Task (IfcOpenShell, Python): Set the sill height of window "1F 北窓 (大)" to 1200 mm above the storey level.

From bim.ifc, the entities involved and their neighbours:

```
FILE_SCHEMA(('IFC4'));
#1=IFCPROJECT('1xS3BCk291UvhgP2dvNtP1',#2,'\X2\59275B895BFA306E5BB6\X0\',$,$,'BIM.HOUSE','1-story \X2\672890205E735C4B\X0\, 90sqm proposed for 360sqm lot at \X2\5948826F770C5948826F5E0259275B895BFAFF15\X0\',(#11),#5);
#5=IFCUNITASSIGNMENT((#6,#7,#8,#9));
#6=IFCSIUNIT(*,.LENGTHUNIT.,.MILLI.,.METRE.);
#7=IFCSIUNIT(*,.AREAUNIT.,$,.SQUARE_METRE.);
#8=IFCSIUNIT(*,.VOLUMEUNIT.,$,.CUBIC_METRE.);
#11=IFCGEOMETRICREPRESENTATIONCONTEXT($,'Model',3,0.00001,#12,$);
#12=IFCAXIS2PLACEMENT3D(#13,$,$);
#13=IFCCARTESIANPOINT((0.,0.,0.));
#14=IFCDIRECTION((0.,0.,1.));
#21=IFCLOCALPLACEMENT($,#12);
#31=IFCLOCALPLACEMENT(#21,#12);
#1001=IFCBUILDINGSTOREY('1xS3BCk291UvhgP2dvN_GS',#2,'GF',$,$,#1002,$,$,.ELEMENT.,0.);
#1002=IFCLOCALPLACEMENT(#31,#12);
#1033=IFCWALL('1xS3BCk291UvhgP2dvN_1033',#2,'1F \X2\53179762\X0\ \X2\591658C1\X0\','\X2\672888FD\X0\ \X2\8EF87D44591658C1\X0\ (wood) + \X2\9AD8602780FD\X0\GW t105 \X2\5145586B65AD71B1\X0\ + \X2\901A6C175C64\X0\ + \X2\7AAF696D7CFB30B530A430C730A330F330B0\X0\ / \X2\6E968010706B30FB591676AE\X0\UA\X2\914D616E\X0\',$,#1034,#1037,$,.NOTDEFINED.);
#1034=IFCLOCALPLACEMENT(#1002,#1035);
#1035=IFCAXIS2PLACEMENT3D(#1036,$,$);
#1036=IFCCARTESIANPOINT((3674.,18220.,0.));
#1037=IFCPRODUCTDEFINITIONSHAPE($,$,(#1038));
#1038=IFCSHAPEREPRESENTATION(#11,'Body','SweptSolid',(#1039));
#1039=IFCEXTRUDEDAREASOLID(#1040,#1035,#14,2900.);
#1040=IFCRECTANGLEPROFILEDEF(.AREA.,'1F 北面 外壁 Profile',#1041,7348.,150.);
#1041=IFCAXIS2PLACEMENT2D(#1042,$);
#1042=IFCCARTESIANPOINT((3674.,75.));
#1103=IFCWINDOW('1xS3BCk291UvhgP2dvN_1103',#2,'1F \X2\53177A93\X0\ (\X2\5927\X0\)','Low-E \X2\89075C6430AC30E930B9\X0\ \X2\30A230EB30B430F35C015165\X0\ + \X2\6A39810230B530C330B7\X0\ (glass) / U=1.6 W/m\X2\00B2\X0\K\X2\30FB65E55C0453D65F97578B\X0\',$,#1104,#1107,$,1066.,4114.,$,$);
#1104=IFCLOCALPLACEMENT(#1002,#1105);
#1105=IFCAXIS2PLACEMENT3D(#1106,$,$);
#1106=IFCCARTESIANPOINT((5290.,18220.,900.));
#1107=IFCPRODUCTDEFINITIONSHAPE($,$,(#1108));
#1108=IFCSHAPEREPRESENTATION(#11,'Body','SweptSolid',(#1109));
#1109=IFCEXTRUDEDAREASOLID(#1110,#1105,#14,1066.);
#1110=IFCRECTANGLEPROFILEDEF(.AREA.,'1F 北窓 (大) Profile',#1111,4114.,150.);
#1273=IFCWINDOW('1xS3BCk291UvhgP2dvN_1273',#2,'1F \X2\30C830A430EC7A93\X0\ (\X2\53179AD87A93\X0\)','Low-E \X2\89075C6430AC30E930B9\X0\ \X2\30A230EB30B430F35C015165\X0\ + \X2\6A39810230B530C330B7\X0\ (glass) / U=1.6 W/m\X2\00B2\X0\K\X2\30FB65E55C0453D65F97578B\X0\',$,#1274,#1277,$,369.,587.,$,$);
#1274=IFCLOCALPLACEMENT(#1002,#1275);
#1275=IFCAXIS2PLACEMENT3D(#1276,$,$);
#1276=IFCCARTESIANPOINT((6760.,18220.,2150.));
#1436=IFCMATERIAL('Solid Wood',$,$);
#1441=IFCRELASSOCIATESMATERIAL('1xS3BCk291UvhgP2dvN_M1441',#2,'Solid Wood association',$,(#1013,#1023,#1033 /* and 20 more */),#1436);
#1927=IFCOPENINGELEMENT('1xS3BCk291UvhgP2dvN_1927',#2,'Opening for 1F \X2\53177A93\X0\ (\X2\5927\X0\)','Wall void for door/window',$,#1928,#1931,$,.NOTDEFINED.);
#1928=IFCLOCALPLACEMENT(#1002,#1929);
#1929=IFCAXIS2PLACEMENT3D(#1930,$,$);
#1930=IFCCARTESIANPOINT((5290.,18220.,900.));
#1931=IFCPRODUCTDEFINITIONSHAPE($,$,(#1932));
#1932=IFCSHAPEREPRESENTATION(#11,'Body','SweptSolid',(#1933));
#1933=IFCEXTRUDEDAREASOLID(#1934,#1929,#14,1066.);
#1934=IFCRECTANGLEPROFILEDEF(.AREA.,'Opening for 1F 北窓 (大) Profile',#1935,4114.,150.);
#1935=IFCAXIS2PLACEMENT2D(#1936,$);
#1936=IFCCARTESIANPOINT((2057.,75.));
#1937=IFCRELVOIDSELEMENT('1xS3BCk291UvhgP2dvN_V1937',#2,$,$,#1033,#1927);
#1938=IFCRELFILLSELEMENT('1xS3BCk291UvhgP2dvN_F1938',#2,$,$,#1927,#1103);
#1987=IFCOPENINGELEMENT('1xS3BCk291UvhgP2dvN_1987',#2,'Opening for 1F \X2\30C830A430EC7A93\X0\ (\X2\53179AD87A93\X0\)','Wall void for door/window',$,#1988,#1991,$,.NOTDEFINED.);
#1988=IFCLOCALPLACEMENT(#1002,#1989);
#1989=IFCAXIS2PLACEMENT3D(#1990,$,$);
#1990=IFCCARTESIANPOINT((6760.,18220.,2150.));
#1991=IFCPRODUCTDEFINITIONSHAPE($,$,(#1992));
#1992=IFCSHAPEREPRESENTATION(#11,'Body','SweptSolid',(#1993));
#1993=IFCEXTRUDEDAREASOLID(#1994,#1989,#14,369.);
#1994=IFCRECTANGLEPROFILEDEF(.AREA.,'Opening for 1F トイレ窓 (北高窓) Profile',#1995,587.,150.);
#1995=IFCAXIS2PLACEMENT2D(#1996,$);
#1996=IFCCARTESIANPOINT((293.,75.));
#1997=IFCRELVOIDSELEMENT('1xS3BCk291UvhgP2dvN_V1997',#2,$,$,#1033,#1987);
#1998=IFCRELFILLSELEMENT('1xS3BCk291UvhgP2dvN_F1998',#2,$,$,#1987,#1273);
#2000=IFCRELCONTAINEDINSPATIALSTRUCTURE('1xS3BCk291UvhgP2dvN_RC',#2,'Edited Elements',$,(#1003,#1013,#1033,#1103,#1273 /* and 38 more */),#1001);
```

```python
import numpy as np
import ifcopenshell
import ifcopenshell.api.geometry
import ifcopenshell.geom
import ifcopenshell.util.element
import ifcopenshell.util.placement
import ifcopenshell.util.shape
import ifcopenshell.util.unit

model = ifcopenshell.open("bim.ifc")
unit_scale = ifcopenshell.util.unit.calculate_unit_scale(model)

window = model.by_guid("1xS3BCk291UvhgP2dvN_1103")
opening = window.FillsVoids[0].RelatingOpeningElement
storey = ifcopenshell.util.element.get_container(window, ifc_class="IfcBuildingStorey")
level = ifcopenshell.util.placement.get_local_placement(storey.ObjectPlacement)[2, 3]

# The opening's origin need not be at the sill, so measure its lowest point.
shape = ifcopenshell.geom.create_shape(ifcopenshell.geom.settings(), opening)
bottom = ifcopenshell.util.shape.get_shape_bottom_elevation(shape, shape.geometry) / unit_scale
dz = level + 1.2 / unit_scale - bottom

shift = np.array([0.0, 0.0, dz])
# The window is not placed relative to its opening, so move both.
for product in (opening, window):
    matrix = ifcopenshell.util.placement.get_local_placement(product.ObjectPlacement)
    matrix[:3, 3] += shift
    ifcopenshell.api.geometry.edit_object_placement(model, product=product, matrix=matrix, is_si=False)

print(f"moved by {dz * unit_scale:+.3f} m")

model.write("bim-out.ifc")
```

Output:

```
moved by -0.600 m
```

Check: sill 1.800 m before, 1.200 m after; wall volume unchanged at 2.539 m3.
